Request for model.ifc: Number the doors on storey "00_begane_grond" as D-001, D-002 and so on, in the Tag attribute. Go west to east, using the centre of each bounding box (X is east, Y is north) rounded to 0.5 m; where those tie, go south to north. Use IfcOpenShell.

First a look at what the model holds.

```python
import ifcopenshell
import ifcopenshell.util.element
import ifcopenshell.util.placement

model = ifcopenshell.open("model.ifc")
print(model.schema)
storey = next(s for s in model.by_type("IfcBuildingStorey") if s.Name == "00_begane_grond")
doors = [e for e in ifcopenshell.util.element.get_decomposition(storey) if e.is_a("IfcDoor")]
for e in sorted(doors, key=lambda e: e.id()):
    origin = ifcopenshell.util.placement.get_local_placement(e.ObjectPlacement)[:3, 3]
    print(e.id(), e.Tag, e.Name, origin.round(2) + 0.0, sep=" | ")
```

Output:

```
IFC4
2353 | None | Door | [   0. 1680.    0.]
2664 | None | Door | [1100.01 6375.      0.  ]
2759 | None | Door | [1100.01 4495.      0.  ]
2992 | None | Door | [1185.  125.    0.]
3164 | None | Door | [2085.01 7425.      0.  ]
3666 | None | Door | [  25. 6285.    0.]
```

```python
import ifcopenshell
import ifcopenshell.geom
import ifcopenshell.util.element
import ifcopenshell.util.shape

model = ifcopenshell.open("model.ifc")
settings = ifcopenshell.geom.settings()
settings.set("use-world-coords", True)


def centre(element):
    shape = ifcopenshell.geom.create_shape(settings, element)
    return ifcopenshell.util.shape.get_bbox_centroid(shape.geometry)


storey = next(s for s in model.by_type("IfcBuildingStorey") if s.Name == "00_begane_grond")
doors = [e for e in ifcopenshell.util.element.get_decomposition(storey) if e.is_a("IfcDoor")]

# Insertion points can sit at a corner or the storey origin, so sort by the geometry (in metres).
centres = {e: centre(e) for e in doors}
doors.sort(key=lambda e: (round(centres[e][0] / 0.5), centres[e][1]))

for i, e in enumerate(doors, start=1):
    number = f"D-0{i:02d}"
    e.Tag = number
    print(e.id(), number)

model.write("model_updated.ifc")
```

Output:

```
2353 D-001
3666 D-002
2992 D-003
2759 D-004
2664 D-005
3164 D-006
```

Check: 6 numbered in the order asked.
